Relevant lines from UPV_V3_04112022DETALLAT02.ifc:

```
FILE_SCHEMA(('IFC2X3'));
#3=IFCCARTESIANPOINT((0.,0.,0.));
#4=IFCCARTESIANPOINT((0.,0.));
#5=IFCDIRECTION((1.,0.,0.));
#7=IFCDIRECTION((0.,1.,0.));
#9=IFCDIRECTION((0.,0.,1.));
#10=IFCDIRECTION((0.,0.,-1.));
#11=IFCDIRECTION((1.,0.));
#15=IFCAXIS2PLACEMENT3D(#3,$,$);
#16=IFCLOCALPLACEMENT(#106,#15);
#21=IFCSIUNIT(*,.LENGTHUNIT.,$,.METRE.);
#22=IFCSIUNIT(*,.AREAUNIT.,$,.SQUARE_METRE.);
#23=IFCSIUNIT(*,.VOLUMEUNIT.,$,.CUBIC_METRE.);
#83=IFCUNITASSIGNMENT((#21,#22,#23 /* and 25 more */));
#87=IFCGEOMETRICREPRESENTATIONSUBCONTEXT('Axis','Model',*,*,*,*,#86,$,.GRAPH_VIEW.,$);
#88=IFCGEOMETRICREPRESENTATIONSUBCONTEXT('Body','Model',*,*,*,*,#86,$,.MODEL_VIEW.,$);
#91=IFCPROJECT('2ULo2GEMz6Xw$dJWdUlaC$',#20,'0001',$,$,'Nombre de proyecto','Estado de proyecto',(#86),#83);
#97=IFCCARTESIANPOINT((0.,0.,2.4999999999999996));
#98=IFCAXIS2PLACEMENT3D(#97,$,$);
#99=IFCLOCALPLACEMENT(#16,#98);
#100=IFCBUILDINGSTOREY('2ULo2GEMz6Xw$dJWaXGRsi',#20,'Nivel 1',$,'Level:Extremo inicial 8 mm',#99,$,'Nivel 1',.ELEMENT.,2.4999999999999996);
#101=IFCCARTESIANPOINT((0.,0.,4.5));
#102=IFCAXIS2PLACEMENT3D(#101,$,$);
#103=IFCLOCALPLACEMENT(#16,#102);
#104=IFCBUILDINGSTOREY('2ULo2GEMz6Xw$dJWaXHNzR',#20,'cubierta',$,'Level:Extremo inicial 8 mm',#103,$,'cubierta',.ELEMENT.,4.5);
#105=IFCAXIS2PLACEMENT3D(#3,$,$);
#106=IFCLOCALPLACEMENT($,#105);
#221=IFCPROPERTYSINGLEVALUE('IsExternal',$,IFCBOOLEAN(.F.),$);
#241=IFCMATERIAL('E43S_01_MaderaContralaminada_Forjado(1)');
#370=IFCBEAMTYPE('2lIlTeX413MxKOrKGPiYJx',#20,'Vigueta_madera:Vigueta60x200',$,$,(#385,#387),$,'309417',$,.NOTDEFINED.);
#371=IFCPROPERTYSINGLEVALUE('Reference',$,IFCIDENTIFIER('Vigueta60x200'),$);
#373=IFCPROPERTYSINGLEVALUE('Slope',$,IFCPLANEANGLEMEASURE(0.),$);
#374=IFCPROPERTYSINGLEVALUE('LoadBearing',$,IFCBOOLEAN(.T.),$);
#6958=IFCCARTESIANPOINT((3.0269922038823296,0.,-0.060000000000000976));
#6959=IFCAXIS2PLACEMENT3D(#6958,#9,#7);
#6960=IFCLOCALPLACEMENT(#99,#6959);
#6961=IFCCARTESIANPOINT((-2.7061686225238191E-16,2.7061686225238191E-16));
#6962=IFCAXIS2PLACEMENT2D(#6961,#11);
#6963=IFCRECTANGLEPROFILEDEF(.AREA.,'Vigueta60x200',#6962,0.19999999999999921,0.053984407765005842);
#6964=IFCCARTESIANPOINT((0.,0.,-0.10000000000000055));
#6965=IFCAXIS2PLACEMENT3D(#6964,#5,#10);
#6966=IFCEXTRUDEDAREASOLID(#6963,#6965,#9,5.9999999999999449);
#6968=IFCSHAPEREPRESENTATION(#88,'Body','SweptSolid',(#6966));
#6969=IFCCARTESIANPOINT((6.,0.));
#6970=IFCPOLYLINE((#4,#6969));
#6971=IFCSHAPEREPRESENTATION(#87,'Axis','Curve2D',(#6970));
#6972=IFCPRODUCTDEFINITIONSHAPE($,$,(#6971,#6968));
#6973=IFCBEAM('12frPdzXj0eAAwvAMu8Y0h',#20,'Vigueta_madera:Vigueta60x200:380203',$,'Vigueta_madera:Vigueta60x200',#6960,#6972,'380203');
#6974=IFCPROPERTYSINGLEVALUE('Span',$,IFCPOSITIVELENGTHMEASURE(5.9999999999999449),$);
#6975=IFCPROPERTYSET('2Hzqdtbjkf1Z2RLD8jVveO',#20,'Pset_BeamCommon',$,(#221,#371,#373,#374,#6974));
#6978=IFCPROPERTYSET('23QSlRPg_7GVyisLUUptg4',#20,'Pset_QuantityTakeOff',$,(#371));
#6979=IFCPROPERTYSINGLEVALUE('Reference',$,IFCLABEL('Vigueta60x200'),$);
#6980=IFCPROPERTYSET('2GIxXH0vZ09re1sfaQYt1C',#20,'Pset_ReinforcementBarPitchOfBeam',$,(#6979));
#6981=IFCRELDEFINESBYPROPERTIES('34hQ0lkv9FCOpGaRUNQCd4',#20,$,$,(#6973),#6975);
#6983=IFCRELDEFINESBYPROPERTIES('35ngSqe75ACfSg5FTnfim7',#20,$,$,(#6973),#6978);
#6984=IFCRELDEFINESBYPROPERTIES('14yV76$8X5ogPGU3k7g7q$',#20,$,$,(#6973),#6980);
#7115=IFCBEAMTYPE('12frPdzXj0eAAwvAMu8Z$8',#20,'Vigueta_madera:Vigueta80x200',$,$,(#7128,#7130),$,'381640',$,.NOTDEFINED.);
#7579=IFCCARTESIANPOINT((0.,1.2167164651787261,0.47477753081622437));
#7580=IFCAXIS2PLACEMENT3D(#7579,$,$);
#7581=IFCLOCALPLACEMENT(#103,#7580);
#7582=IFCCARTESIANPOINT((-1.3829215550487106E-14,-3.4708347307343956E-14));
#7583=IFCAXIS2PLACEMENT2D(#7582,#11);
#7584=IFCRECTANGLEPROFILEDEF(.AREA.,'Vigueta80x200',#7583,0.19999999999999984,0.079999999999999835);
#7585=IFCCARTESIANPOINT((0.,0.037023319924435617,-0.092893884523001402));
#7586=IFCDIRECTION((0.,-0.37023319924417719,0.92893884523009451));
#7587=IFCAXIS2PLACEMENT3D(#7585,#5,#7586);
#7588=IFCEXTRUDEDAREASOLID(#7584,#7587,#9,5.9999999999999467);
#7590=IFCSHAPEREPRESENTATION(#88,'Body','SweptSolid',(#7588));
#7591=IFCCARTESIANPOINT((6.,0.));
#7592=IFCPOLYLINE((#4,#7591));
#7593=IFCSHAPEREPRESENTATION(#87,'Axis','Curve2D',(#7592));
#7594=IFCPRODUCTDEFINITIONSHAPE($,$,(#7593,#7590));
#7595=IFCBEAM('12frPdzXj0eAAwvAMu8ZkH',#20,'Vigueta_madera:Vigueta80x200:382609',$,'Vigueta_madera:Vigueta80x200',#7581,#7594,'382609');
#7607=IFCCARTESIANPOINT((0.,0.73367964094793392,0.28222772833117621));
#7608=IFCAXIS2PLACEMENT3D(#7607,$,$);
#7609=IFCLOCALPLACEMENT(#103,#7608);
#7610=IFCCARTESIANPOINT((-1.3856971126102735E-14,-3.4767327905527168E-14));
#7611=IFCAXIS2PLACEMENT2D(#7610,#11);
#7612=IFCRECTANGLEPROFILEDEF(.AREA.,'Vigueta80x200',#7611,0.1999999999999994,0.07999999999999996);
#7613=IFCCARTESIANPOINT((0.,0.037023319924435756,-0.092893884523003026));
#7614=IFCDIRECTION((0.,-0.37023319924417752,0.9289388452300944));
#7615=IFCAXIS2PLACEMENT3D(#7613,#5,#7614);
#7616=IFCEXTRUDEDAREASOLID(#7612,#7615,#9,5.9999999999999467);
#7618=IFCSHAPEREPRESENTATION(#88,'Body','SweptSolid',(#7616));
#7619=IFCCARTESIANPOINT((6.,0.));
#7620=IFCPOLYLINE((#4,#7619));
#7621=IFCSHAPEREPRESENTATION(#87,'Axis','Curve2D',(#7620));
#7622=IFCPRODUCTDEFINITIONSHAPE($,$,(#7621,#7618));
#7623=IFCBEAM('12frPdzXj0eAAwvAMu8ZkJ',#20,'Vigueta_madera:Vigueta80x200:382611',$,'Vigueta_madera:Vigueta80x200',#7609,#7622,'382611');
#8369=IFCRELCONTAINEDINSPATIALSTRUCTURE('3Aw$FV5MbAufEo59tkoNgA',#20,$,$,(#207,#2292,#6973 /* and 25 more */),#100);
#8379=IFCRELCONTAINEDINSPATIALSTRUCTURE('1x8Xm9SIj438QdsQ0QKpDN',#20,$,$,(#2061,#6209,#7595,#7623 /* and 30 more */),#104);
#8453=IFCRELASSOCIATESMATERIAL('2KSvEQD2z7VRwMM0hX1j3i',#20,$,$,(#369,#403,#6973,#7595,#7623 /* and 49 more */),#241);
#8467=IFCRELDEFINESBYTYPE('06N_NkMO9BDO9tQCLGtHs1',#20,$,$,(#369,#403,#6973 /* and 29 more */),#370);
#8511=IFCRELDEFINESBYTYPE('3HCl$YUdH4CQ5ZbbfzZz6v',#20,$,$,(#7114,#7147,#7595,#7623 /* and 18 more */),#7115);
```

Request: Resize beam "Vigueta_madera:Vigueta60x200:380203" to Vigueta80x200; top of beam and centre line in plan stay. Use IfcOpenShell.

```python
import ifcopenshell
import ifcopenshell.api.pset
import ifcopenshell.api.type
import ifcopenshell.util.element
import ifcopenshell.util.representation

model = ifcopenshell.open("UPV_V3_04112022DETALLAT02.ifc")

member = model.by_id(6973)
source = next(p for p in model.by_type("IfcRectangleProfileDef") if p.ProfileName == "Vigueta80x200")

body = ifcopenshell.util.representation.get_representation(member, "Model", "Body")
solid = body.Items[0]
old_profile = solid.SweptArea

# Copy the section's sizes but keep this member's own profile position.
profile = ifcopenshell.util.element.copy(model, source)
# Profiles are centred, so shift by half the change in depth to hold the top.
shift = (old_profile.XDim - profile.XDim) / 2
x, y = old_profile.Position.Location.Coordinates
up = (-1.0, 0.0)  # upwards, in the solid's own plane
location = model.createIfcCartesianPoint((x + up[0] * shift, y + up[1] * shift))
profile.Position = model.createIfcAxis2Placement2D(location, old_profile.Position.RefDirection)
solid.SweptArea = profile
if not model.get_total_inverses(old_profile):
    ifcopenshell.util.element.remove_deep2(model, old_profile)

new_type = model.by_id(7115)
ifcopenshell.api.type.assign_type(
    model, related_objects=[member], relating_type=new_type, should_map_representations=False
)
member.Name = member.Name.replace("Vigueta60x200", "Vigueta80x200")
member.ObjectType = "Vigueta_madera:Vigueta80x200"
pset = model.by_id(ifcopenshell.util.element.get_pset(member, "Pset_BeamCommon", should_inherit=False)["id"])
ifcopenshell.api.pset.edit_pset(model, pset=pset, properties={"Reference": "Vigueta80x200"})
pset = model.by_id(ifcopenshell.util.element.get_pset(member, "Pset_QuantityTakeOff", should_inherit=False)["id"])
ifcopenshell.api.pset.edit_pset(model, pset=pset, properties={"Reference": "Vigueta80x200"})
pset = model.by_id(ifcopenshell.util.element.get_pset(member, "Pset_ReinforcementBarPitchOfBeam", should_inherit=False)["id"])
ifcopenshell.api.pset.edit_pset(model, pset=pset, properties={"Reference": "Vigueta80x200"})

print(solid.SweptArea)

model.write("UPV_V3_04112022DETALLAT02_rev.ifc")
```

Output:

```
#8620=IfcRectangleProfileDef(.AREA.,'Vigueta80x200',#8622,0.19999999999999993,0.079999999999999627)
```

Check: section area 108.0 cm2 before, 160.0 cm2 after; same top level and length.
